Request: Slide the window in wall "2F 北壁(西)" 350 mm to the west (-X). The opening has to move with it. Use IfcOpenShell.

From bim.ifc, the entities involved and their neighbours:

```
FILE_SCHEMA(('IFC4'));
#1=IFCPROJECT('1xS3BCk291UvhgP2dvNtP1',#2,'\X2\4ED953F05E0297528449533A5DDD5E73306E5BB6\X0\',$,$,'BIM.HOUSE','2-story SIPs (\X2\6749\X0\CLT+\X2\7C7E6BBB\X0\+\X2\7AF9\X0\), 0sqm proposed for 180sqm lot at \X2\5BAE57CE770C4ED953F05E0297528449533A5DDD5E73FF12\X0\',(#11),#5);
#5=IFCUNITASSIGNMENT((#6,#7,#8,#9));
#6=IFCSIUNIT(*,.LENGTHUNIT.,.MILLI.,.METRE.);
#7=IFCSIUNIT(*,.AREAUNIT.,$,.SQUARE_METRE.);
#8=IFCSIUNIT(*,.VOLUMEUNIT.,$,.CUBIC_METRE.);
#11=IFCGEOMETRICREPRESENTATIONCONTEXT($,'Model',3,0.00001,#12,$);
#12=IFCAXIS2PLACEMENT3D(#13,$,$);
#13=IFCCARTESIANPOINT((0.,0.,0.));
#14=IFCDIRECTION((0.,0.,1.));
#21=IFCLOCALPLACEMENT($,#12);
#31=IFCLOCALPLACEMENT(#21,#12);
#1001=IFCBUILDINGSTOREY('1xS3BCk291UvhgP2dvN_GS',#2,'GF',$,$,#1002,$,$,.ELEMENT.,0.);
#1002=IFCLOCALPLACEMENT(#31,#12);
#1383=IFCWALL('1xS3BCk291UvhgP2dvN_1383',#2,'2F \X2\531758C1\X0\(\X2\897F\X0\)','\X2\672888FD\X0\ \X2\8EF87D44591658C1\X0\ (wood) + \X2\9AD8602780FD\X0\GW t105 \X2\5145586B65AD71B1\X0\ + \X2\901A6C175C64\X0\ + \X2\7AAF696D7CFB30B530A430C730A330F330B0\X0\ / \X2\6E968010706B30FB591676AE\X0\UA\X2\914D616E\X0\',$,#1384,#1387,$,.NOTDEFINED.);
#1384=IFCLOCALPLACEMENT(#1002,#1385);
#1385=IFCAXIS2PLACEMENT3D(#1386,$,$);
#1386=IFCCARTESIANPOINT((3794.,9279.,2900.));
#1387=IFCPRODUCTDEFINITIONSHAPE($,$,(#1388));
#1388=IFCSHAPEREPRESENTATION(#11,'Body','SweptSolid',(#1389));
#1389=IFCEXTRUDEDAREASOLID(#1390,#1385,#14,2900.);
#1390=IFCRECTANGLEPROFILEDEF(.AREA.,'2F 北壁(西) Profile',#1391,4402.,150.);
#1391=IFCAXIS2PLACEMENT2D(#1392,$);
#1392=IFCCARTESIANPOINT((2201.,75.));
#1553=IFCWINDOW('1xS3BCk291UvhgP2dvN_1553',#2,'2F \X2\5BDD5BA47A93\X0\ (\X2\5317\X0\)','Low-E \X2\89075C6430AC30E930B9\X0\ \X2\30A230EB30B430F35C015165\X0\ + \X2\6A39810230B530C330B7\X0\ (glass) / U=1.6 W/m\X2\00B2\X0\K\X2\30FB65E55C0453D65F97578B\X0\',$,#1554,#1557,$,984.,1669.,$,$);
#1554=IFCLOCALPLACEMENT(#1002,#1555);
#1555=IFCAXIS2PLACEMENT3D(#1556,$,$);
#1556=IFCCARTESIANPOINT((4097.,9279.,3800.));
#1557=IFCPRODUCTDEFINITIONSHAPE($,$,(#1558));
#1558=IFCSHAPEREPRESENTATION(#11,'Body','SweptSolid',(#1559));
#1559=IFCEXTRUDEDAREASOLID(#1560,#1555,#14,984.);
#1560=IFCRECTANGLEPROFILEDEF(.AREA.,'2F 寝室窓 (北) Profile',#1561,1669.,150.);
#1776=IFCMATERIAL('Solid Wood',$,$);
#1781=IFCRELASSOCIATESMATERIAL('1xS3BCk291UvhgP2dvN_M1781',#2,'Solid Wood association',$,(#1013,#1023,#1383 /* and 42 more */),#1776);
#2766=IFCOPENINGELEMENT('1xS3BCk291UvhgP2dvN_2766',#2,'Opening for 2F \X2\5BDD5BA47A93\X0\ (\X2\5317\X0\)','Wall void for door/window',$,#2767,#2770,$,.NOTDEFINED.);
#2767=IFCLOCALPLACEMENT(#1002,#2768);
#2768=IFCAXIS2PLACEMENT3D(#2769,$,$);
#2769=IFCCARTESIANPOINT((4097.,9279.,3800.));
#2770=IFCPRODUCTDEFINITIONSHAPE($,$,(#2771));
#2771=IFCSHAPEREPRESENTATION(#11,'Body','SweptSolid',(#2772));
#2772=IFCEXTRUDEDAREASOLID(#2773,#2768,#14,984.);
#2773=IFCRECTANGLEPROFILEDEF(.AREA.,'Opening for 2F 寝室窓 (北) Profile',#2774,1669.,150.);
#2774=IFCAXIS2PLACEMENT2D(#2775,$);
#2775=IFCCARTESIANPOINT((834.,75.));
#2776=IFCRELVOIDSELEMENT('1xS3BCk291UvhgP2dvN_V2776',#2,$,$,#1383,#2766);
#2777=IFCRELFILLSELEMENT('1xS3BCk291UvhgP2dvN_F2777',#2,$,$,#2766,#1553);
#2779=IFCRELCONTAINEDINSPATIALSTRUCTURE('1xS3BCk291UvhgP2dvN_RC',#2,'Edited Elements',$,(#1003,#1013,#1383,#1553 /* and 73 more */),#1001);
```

```python
import ifcopenshell
import ifcopenshell.api.geometry
import ifcopenshell.util.placement
import ifcopenshell.util.unit

model = ifcopenshell.open("bim.ifc")
unit_scale = ifcopenshell.util.unit.calculate_unit_scale(model)

window = model.by_id(1553)
opening = window.FillsVoids[0].RelatingOpeningElement
wall = opening.VoidsElements[0].RelatingBuildingElement

wall_matrix = ifcopenshell.util.placement.get_local_placement(wall.ObjectPlacement)
shift = wall_matrix[:3, 0] * -0.35 / unit_scale
before = ifcopenshell.util.placement.get_local_placement(window.ObjectPlacement)[:3, 3].copy()

# The window is not placed relative to its opening, so move both.
for product in (opening, window):
    matrix = ifcopenshell.util.placement.get_local_placement(product.ObjectPlacement)
    matrix[:3, 3] += shift
    ifcopenshell.api.geometry.edit_object_placement(model, product=product, matrix=matrix, is_si=False)

after = ifcopenshell.util.placement.get_local_placement(window.ObjectPlacement)[:3, 3]
print("window moved by", (after - before).round(3) + 0.0)

model.write("bim_rev.ifc")
```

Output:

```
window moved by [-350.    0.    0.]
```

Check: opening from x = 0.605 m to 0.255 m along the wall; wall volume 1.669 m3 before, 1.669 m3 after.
